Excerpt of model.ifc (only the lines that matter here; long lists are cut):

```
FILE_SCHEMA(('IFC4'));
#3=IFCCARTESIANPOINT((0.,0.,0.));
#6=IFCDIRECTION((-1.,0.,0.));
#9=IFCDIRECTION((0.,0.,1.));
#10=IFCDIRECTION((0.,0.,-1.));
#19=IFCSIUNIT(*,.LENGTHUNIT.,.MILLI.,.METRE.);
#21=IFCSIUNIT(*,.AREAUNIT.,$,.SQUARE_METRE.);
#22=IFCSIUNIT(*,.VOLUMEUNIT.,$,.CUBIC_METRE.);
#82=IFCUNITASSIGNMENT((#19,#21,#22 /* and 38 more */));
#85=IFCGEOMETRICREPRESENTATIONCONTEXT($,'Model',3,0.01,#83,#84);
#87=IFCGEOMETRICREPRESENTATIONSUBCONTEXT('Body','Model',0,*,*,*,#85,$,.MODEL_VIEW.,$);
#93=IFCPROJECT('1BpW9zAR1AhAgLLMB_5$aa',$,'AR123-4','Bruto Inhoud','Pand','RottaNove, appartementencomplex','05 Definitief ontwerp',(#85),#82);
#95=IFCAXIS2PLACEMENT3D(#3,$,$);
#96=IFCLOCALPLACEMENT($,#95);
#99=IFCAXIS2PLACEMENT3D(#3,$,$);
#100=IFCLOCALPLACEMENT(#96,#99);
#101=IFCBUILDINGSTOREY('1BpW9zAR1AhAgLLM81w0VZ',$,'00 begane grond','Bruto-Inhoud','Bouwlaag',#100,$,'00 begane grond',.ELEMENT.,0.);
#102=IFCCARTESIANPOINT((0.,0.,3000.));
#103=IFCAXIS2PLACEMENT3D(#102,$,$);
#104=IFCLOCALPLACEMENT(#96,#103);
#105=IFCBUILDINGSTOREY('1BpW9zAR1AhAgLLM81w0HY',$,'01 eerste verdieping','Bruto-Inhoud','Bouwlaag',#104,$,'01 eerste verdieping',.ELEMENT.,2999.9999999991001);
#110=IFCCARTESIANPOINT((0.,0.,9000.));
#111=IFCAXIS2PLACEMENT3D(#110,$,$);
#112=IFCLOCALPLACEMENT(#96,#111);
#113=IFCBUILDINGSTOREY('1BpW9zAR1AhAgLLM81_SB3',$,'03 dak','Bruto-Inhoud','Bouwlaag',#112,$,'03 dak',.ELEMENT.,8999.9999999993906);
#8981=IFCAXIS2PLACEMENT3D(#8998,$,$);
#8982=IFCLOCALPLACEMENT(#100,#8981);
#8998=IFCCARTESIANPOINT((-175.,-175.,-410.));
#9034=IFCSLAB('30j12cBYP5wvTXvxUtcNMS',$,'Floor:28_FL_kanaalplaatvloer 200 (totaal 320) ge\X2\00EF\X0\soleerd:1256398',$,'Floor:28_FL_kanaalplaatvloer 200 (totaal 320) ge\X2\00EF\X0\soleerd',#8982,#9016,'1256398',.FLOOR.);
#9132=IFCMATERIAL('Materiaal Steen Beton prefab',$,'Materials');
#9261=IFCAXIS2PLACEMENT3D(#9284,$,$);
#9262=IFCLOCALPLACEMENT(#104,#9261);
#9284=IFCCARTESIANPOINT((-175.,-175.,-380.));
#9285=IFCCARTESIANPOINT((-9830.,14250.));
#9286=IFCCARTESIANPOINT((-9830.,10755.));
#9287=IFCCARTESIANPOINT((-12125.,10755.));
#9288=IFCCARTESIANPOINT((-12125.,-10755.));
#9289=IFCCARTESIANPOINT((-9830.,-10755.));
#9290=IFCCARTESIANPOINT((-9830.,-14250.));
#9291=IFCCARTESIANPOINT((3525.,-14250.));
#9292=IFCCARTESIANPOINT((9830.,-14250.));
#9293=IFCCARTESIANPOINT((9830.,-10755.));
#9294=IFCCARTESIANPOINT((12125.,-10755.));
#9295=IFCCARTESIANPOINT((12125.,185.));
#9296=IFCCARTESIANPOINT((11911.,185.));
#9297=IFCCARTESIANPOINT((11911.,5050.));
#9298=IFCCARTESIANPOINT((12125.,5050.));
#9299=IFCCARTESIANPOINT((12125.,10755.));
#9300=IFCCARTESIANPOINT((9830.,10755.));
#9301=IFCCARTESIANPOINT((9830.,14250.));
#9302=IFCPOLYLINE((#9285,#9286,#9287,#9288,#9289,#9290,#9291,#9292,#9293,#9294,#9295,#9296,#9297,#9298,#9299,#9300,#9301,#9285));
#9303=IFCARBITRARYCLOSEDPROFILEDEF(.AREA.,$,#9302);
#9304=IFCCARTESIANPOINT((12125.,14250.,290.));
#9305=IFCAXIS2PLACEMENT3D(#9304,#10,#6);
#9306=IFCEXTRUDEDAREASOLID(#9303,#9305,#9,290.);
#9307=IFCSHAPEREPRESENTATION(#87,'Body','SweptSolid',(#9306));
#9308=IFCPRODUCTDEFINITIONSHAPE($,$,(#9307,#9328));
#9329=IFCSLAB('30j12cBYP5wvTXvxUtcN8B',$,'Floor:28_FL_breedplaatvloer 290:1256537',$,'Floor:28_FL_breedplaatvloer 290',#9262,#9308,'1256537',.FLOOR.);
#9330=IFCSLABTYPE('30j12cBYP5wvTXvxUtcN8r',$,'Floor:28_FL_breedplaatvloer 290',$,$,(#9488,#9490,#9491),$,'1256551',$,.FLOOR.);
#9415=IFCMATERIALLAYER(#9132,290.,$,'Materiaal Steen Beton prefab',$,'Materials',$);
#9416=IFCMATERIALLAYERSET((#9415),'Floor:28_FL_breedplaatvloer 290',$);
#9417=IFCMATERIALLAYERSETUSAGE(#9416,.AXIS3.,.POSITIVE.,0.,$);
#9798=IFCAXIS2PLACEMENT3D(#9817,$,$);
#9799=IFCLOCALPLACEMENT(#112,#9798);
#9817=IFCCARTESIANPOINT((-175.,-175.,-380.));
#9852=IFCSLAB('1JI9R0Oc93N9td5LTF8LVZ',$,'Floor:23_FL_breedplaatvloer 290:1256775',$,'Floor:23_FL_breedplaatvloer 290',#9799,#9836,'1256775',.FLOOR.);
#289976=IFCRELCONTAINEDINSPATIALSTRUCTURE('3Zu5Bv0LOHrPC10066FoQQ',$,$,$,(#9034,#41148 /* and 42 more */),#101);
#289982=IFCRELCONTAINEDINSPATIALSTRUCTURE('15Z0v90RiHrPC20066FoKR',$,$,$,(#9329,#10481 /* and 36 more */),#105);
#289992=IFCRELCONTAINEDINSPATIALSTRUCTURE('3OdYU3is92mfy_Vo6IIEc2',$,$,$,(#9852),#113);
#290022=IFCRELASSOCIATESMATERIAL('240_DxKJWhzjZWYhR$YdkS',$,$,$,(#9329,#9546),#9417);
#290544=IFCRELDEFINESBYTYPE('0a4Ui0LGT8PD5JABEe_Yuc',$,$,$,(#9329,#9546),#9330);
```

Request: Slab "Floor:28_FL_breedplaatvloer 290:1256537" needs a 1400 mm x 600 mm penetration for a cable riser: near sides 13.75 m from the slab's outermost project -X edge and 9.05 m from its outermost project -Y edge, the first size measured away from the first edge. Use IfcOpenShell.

```python
import numpy as np
import ifcopenshell
import ifcopenshell.api.feature
import ifcopenshell.api.geometry
import ifcopenshell.api.root
import ifcopenshell.geom
import ifcopenshell.util.placement
import ifcopenshell.util.representation
import ifcopenshell.util.shape
import ifcopenshell.util.unit

model = ifcopenshell.open("model.ifc")
unit_scale = ifcopenshell.util.unit.calculate_unit_scale(model)
settings = ifcopenshell.geom.settings()


def volume(element):
    """Net volume in cubic metres, openings subtracted."""
    shape = ifcopenshell.geom.create_shape(settings, element)
    return ifcopenshell.util.shape.get_volume(shape.geometry)


slab = model.by_guid("30j12cBYP5wvTXvxUtcN8B")
before = volume(slab)

# Extent in the slab's own axes, in metres. The edges named are its -X and -Y sides.
slab_shape = ifcopenshell.geom.create_shape(settings, slab)
vertices = ifcopenshell.util.shape.get_vertices(slab_shape.geometry)
x_min, y_min, bottom = vertices.min(axis=0)
top = vertices[:, 2].max()

opening = ifcopenshell.api.root.create_entity(model, ifc_class="IfcOpeningElement", name="Cable riser opening", predefined_type="OPENING")
context = ifcopenshell.util.representation.get_context(model, "Model", "Body", "MODEL_VIEW")
width, depth = 1.4, 0.6
outline = [(0.0, 0.0), (width, 0.0), (width, depth), (0.0, depth), (0.0, 0.0)]
# Overshoot both faces by 50 mm so the cut is clean.
shape = ifcopenshell.api.geometry.add_slab_representation(
    model, context=context, depth=top - bottom + 0.1, polyline=outline
)
ifcopenshell.api.geometry.assign_representation(model, product=opening, representation=shape)

matrix = ifcopenshell.util.placement.get_local_placement(slab.ObjectPlacement)
matrix[:, 3] = matrix @ np.append(np.array([x_min + 13.75, y_min + 9.05, bottom - 0.05]) / unit_scale, 1.0)
ifcopenshell.api.geometry.edit_object_placement(model, product=opening, matrix=matrix, is_si=False)
ifcopenshell.api.feature.add_feature(model, feature=opening, element=slab)

after = volume(slab)

print(f"slab volume {before:.3f} -> {after:.3f} m3")

model.write("model_v2.ifc")
```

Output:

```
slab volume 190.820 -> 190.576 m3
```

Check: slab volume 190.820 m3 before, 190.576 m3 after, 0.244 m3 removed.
